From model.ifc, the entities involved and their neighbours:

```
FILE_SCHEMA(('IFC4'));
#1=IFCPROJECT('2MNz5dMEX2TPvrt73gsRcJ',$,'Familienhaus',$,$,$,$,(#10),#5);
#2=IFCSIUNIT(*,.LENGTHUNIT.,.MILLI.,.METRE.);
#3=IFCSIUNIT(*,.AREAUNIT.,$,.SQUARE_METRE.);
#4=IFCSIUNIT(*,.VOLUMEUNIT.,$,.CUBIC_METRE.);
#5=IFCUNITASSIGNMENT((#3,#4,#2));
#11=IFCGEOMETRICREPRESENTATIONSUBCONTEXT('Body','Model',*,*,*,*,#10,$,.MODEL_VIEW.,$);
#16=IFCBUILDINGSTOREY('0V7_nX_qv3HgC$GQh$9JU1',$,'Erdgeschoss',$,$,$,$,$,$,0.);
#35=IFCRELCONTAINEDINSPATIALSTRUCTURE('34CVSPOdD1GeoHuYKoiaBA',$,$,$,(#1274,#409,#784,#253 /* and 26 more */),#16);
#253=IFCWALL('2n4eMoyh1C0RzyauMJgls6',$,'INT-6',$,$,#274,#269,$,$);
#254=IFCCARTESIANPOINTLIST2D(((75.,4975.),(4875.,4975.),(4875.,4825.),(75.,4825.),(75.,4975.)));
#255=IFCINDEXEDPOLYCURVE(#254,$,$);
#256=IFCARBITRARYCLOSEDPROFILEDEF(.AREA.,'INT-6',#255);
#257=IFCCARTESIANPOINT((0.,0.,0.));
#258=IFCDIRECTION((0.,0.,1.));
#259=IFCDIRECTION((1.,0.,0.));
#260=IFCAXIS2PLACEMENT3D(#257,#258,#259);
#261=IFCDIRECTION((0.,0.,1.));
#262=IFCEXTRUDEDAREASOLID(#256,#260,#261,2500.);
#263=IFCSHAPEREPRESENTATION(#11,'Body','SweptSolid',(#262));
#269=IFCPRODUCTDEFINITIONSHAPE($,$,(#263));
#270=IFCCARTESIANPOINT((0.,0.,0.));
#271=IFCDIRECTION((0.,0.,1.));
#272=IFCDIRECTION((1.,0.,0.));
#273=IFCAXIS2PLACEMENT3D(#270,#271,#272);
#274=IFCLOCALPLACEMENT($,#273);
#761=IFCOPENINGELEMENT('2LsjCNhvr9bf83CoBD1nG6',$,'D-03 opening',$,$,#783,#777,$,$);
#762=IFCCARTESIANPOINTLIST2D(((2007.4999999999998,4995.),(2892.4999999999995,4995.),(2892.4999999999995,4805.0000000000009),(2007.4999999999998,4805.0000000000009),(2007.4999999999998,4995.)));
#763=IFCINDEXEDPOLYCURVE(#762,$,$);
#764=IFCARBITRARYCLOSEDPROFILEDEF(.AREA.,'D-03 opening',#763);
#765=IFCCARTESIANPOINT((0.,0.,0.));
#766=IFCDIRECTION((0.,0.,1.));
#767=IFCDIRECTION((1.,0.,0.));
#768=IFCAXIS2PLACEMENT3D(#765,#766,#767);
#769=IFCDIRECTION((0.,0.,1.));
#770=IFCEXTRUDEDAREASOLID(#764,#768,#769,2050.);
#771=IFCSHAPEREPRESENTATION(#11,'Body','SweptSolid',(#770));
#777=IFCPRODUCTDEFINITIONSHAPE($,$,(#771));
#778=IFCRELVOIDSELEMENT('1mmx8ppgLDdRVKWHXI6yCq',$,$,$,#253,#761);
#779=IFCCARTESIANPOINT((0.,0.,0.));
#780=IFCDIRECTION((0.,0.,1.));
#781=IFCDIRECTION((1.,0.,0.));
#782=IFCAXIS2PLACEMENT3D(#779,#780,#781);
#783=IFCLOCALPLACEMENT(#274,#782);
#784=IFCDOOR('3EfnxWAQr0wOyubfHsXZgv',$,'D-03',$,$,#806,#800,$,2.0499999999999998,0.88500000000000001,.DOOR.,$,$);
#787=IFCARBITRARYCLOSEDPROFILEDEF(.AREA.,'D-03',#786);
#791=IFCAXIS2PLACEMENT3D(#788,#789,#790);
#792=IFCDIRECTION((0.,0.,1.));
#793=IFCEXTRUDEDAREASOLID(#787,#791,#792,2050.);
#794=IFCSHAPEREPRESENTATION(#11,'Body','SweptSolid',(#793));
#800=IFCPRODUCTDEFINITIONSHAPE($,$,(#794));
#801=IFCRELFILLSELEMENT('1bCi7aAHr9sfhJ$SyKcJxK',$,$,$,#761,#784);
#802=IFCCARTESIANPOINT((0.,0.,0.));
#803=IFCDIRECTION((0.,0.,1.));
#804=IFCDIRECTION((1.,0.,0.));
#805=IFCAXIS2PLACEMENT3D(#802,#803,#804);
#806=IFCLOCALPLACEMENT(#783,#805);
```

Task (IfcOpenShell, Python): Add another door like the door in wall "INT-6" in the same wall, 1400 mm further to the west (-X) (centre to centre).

```python
import ifcopenshell
import ifcopenshell.api.feature
import ifcopenshell.api.geometry
import ifcopenshell.api.root
import ifcopenshell.geom
import ifcopenshell.util.element
import ifcopenshell.util.placement
import ifcopenshell.util.shape
import ifcopenshell.util.unit

model = ifcopenshell.open("model.ifc")
unit_scale = ifcopenshell.util.unit.calculate_unit_scale(model)
settings = ifcopenshell.geom.settings()


def volume(element):
    """Net volume in cubic metres, openings subtracted."""
    shape = ifcopenshell.geom.create_shape(settings, element)
    return ifcopenshell.util.shape.get_volume(shape.geometry)


door = model.by_guid("3EfnxWAQr0wOyubfHsXZgv")
opening = door.FillsVoids[0].RelatingOpeningElement
wall = opening.VoidsElements[0].RelatingBuildingElement
before = volume(wall)
shift = ifcopenshell.util.placement.get_local_placement(wall.ObjectPlacement)[:3, 0] * -1.4 / unit_scale

# copy_class copies the void relationship, type, container and properties, but no geometry.
new_opening = ifcopenshell.api.root.copy_class(model, product=opening)
new_opening.Representation = ifcopenshell.util.element.copy_deep(
    model, opening.Representation, exclude=["IfcGeometricRepresentationContext", "IfcRepresentationMap"]
)
new_door = ifcopenshell.api.root.copy_class(model, product=door)
new_door.Representation = ifcopenshell.util.element.copy_deep(
    model, door.Representation, exclude=["IfcGeometricRepresentationContext", "IfcRepresentationMap"]
)
ifcopenshell.api.feature.add_filling(model, opening=new_opening, element=new_door)

for old, new in ((opening, new_opening), (door, new_door)):
    matrix = ifcopenshell.util.placement.get_local_placement(old.ObjectPlacement)
    matrix[:3, 3] += shift
    ifcopenshell.api.geometry.edit_object_placement(model, product=new, matrix=matrix, is_si=False)

after = volume(wall)

print(f"wall volume {before:.3f} -> {after:.3f} m3")

model.write("model_updated.ifc")
```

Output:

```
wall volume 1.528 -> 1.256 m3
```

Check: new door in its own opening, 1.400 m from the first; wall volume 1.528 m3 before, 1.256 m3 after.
